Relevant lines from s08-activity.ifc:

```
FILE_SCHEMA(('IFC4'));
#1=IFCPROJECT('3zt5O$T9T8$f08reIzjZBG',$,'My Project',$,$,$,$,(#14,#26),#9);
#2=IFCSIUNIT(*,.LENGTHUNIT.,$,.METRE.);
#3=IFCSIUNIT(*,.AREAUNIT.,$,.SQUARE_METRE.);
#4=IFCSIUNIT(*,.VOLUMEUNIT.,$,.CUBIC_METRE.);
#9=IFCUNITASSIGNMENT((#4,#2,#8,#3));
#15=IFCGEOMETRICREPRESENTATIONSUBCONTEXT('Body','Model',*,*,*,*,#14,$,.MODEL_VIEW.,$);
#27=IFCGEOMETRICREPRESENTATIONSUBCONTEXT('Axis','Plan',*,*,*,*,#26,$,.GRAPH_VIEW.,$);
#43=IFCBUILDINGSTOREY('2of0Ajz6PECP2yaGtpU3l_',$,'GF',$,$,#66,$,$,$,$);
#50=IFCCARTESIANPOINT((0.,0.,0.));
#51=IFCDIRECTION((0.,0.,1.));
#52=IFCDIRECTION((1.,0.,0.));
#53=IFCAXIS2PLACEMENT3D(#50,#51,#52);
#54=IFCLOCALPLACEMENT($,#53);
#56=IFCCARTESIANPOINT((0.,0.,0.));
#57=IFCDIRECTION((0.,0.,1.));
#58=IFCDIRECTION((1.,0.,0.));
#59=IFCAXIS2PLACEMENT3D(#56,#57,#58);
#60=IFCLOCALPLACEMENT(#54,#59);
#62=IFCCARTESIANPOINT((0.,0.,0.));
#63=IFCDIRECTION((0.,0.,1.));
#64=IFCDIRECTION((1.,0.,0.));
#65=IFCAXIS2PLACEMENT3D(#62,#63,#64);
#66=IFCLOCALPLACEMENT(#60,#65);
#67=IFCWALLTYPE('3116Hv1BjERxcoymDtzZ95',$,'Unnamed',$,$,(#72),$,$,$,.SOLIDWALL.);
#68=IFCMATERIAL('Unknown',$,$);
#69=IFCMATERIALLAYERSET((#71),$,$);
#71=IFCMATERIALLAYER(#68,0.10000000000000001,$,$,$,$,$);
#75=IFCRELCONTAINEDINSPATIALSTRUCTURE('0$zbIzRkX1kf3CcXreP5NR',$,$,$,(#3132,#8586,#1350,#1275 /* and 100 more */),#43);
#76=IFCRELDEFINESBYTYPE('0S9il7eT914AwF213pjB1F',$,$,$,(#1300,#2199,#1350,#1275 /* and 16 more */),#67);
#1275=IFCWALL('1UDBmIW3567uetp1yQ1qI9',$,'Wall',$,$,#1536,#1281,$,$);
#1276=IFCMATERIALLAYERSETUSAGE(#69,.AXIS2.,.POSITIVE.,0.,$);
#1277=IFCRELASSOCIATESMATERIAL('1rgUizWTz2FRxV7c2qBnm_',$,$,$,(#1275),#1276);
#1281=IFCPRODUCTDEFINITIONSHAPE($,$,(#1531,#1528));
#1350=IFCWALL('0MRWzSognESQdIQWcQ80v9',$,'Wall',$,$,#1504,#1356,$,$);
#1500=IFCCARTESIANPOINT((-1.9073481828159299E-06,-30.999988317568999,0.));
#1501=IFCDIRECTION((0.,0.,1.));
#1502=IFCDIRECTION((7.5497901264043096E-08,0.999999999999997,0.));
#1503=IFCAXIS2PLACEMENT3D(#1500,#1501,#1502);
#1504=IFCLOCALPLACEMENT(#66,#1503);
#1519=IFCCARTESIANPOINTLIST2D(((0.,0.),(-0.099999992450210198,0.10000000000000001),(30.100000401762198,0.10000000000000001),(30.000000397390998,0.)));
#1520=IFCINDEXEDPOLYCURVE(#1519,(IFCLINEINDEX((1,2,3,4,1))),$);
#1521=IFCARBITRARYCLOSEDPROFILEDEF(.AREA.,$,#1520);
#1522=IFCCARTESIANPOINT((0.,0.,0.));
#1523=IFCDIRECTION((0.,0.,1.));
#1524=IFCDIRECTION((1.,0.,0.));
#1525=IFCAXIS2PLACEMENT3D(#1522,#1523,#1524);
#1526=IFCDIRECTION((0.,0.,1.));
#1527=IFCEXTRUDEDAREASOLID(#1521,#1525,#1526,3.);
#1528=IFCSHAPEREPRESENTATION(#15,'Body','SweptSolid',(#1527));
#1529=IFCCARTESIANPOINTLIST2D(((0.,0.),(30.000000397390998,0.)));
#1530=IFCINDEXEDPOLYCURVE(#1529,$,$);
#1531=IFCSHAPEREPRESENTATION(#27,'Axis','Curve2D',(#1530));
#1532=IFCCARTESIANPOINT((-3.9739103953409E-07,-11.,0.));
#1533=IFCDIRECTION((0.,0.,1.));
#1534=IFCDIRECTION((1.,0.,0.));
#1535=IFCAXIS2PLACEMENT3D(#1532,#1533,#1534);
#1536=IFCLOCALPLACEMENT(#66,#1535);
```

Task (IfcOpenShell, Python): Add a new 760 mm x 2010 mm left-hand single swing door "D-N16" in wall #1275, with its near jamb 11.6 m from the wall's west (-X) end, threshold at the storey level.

```python
import numpy as np
import ifcopenshell
import ifcopenshell.api.feature
import ifcopenshell.api.geometry
import ifcopenshell.api.root
import ifcopenshell.api.spatial
import ifcopenshell.geom
import ifcopenshell.util.element
import ifcopenshell.util.placement
import ifcopenshell.util.representation
import ifcopenshell.util.shape
import ifcopenshell.util.unit

model = ifcopenshell.open("s08-activity.ifc")
unit_scale = ifcopenshell.util.unit.calculate_unit_scale(model)
settings = ifcopenshell.geom.settings()


def volume(element):
    """Net volume in cubic metres, openings subtracted."""
    shape = ifcopenshell.geom.create_shape(settings, element)
    return ifcopenshell.util.shape.get_volume(shape.geometry)


wall = model.by_guid("1UDBmIW3567uetp1yQ1qI9")
storey = ifcopenshell.util.element.get_container(wall, ifc_class="IfcBuildingStorey")
context = ifcopenshell.util.representation.get_context(model, "Model", "Body", "MODEL_VIEW")
before = volume(wall)

width, height, from_end, sill = 0.76, 2.01, 11.6, 0.0  # metres

# The wall runs along its own X axis, and the end named is its -X end.
wall_shape = ifcopenshell.geom.create_shape(settings, wall)
x, y, z = ifcopenshell.util.shape.get_vertices(wall_shape.geometry).T
start = x.min() + from_end
face, thickness = float(y.min()), float(y.max() - y.min())
wall_matrix = ifcopenshell.util.placement.get_local_placement(wall.ObjectPlacement)
level = ifcopenshell.util.placement.get_local_placement(storey.ObjectPlacement)[2, 3]


def in_wall(x, y):
    """Placement at x, y metres in the wall's axes, at sill height."""
    matrix = wall_matrix.copy()
    matrix[:, 3] = wall_matrix @ np.array([x / unit_scale, y / unit_scale, 0.0, 1.0])
    matrix[2, 3] = level + sill / unit_scale
    return matrix


# Opening: a box that overshoots both wall faces by 50 mm.
opening = ifcopenshell.api.root.create_entity(model, ifc_class="IfcOpeningElement", predefined_type="OPENING")
box = ifcopenshell.api.geometry.add_wall_representation(
    model, context=context, length=width, height=height, thickness=thickness + 0.1
)
ifcopenshell.api.geometry.assign_representation(model, product=opening, representation=box)
ifcopenshell.api.geometry.edit_object_placement(model, product=opening, matrix=in_wall(start, face - 0.05), is_si=False)
ifcopenshell.api.feature.add_feature(model, feature=opening, element=wall)

door = ifcopenshell.api.root.create_entity(model, ifc_class="IfcDoor", name="D-N16", predefined_type="DOOR")
door.OverallWidth, door.OverallHeight = width / unit_scale, height / unit_scale
door.OperationType = "SINGLE_SWING_LEFT"
body = ifcopenshell.api.geometry.add_door_representation(
    model,
    context=context,
    overall_width=door.OverallWidth,
    overall_height=door.OverallHeight,
    operation_type="SINGLE_SWING_LEFT",
    lining_properties={"LiningDepth": thickness / unit_scale, "ThresholdDepth": thickness / unit_scale},
)
ifcopenshell.api.geometry.assign_representation(model, product=door, representation=body)
ifcopenshell.api.spatial.assign_container(model, products=[door], relating_structure=storey)
ifcopenshell.api.feature.add_filling(model, opening=opening, element=door)

# The lining spans the wall, so the door starts at the wall face.
ifcopenshell.api.geometry.edit_object_placement(model, product=door, matrix=in_wall(start, face), is_si=False)

after = volume(wall)

print(f"wall volume {before:.3f} -> {after:.3f} m3")

model.write("s08-activity-out.ifc")
```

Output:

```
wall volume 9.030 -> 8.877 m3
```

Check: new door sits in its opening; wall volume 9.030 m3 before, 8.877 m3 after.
